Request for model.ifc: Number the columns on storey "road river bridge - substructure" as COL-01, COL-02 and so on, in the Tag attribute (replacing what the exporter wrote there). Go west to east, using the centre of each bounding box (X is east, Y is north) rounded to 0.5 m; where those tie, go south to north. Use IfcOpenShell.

First a look at what the model holds.

```python
import ifcopenshell
import ifcopenshell.util.element
import ifcopenshell.util.placement

model = ifcopenshell.open("model.ifc")
print(model.schema)
storey = next(s for s in model.by_type("IfcBuildingStorey") if s.Name == "road river bridge - substructure")
columns = [e for e in ifcopenshell.util.element.get_decomposition(storey) if e.is_a("IfcColumn")]
for e in sorted(columns, key=lambda e: e.id()):
    origin = ifcopenshell.util.placement.get_local_placement(e.ObjectPlacement)[:3, 3]
    print(e.id(), e.Tag, e.Name, origin.round(2) + 0.0, sep=" | ")
```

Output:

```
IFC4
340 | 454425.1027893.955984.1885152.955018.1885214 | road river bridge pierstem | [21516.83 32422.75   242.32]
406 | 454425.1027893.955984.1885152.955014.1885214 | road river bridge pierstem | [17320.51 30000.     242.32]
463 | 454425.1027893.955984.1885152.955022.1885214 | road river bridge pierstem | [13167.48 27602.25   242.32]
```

```python
import ifcopenshell
import ifcopenshell.geom
import ifcopenshell.util.element
import ifcopenshell.util.shape

model = ifcopenshell.open("model.ifc")
settings = ifcopenshell.geom.settings()
settings.set("use-world-coords", True)


def centre(element):
    shape = ifcopenshell.geom.create_shape(settings, element)
    return ifcopenshell.util.shape.get_bbox_centroid(shape.geometry)


storey = next(s for s in model.by_type("IfcBuildingStorey") if s.Name == "road river bridge - substructure")
columns = [e for e in ifcopenshell.util.element.get_decomposition(storey) if e.is_a("IfcColumn")]

# Insertion points can sit at a corner or the storey origin, so sort by the geometry (in metres).
centres = {e: centre(e) for e in columns}
columns.sort(key=lambda e: (round(centres[e][0] / 0.5), centres[e][1]))

for i, e in enumerate(columns, start=1):
    number = f"COL-{i:02d}"
    e.Tag = number
    print(e.id(), number)

model.write("model-out.ifc")
```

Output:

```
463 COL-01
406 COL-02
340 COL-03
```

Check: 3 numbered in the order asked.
